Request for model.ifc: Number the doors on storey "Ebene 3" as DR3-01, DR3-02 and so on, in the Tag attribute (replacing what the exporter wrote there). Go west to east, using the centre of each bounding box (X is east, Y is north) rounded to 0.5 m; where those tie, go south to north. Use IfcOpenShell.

First a look at what the model holds.

```python
import ifcopenshell
import ifcopenshell.util.element
import ifcopenshell.util.placement

model = ifcopenshell.open("model.ifc")
print(model.schema)
storey = next(s for s in model.by_type("IfcBuildingStorey") if s.Name == "Ebene 3")
doors = [e for e in ifcopenshell.util.element.get_decomposition(storey) if e.is_a("IfcDoor")]
for e in sorted(doors, key=lambda e: e.id()):
    origin = ifcopenshell.util.placement.get_local_placement(e.ObjectPlacement)[:3, 3]
    print(e.id(), e.Tag, e.Name, origin.round(2) + 0.0, sep=" | ")
```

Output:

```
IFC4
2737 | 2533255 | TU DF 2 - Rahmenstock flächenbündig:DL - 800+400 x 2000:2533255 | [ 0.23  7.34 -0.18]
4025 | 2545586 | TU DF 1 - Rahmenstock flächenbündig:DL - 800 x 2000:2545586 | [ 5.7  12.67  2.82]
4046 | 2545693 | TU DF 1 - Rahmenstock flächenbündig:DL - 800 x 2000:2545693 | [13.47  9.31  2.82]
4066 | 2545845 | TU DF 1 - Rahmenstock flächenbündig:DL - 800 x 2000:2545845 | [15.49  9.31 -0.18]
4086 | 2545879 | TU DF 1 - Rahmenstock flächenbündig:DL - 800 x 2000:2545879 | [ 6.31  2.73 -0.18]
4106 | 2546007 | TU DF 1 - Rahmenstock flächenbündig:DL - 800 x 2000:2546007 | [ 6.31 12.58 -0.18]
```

```python
import ifcopenshell
import ifcopenshell.geom
import ifcopenshell.util.element
import ifcopenshell.util.shape

model = ifcopenshell.open("model.ifc")
settings = ifcopenshell.geom.settings()
settings.set("use-world-coords", True)


def centre(element):
    shape = ifcopenshell.geom.create_shape(settings, element)
    return ifcopenshell.util.shape.get_bbox_centroid(shape.geometry)


storey = next(s for s in model.by_type("IfcBuildingStorey") if s.Name == "Ebene 3")
doors = [e for e in ifcopenshell.util.element.get_decomposition(storey) if e.is_a("IfcDoor")]

# Insertion points can sit at a corner or the storey origin, so sort by the geometry (in metres).
centres = {e: centre(e) for e in doors}
doors.sort(key=lambda e: (round(centres[e][0] / 0.5), centres[e][1]))

for i, e in enumerate(doors, start=1):
    number = f"DR3-{i:02d}"
    e.Tag = number
    print(e.id(), number)

model.write("model_rev.ifc")
```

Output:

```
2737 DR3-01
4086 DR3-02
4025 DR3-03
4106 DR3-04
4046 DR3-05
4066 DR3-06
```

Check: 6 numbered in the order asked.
